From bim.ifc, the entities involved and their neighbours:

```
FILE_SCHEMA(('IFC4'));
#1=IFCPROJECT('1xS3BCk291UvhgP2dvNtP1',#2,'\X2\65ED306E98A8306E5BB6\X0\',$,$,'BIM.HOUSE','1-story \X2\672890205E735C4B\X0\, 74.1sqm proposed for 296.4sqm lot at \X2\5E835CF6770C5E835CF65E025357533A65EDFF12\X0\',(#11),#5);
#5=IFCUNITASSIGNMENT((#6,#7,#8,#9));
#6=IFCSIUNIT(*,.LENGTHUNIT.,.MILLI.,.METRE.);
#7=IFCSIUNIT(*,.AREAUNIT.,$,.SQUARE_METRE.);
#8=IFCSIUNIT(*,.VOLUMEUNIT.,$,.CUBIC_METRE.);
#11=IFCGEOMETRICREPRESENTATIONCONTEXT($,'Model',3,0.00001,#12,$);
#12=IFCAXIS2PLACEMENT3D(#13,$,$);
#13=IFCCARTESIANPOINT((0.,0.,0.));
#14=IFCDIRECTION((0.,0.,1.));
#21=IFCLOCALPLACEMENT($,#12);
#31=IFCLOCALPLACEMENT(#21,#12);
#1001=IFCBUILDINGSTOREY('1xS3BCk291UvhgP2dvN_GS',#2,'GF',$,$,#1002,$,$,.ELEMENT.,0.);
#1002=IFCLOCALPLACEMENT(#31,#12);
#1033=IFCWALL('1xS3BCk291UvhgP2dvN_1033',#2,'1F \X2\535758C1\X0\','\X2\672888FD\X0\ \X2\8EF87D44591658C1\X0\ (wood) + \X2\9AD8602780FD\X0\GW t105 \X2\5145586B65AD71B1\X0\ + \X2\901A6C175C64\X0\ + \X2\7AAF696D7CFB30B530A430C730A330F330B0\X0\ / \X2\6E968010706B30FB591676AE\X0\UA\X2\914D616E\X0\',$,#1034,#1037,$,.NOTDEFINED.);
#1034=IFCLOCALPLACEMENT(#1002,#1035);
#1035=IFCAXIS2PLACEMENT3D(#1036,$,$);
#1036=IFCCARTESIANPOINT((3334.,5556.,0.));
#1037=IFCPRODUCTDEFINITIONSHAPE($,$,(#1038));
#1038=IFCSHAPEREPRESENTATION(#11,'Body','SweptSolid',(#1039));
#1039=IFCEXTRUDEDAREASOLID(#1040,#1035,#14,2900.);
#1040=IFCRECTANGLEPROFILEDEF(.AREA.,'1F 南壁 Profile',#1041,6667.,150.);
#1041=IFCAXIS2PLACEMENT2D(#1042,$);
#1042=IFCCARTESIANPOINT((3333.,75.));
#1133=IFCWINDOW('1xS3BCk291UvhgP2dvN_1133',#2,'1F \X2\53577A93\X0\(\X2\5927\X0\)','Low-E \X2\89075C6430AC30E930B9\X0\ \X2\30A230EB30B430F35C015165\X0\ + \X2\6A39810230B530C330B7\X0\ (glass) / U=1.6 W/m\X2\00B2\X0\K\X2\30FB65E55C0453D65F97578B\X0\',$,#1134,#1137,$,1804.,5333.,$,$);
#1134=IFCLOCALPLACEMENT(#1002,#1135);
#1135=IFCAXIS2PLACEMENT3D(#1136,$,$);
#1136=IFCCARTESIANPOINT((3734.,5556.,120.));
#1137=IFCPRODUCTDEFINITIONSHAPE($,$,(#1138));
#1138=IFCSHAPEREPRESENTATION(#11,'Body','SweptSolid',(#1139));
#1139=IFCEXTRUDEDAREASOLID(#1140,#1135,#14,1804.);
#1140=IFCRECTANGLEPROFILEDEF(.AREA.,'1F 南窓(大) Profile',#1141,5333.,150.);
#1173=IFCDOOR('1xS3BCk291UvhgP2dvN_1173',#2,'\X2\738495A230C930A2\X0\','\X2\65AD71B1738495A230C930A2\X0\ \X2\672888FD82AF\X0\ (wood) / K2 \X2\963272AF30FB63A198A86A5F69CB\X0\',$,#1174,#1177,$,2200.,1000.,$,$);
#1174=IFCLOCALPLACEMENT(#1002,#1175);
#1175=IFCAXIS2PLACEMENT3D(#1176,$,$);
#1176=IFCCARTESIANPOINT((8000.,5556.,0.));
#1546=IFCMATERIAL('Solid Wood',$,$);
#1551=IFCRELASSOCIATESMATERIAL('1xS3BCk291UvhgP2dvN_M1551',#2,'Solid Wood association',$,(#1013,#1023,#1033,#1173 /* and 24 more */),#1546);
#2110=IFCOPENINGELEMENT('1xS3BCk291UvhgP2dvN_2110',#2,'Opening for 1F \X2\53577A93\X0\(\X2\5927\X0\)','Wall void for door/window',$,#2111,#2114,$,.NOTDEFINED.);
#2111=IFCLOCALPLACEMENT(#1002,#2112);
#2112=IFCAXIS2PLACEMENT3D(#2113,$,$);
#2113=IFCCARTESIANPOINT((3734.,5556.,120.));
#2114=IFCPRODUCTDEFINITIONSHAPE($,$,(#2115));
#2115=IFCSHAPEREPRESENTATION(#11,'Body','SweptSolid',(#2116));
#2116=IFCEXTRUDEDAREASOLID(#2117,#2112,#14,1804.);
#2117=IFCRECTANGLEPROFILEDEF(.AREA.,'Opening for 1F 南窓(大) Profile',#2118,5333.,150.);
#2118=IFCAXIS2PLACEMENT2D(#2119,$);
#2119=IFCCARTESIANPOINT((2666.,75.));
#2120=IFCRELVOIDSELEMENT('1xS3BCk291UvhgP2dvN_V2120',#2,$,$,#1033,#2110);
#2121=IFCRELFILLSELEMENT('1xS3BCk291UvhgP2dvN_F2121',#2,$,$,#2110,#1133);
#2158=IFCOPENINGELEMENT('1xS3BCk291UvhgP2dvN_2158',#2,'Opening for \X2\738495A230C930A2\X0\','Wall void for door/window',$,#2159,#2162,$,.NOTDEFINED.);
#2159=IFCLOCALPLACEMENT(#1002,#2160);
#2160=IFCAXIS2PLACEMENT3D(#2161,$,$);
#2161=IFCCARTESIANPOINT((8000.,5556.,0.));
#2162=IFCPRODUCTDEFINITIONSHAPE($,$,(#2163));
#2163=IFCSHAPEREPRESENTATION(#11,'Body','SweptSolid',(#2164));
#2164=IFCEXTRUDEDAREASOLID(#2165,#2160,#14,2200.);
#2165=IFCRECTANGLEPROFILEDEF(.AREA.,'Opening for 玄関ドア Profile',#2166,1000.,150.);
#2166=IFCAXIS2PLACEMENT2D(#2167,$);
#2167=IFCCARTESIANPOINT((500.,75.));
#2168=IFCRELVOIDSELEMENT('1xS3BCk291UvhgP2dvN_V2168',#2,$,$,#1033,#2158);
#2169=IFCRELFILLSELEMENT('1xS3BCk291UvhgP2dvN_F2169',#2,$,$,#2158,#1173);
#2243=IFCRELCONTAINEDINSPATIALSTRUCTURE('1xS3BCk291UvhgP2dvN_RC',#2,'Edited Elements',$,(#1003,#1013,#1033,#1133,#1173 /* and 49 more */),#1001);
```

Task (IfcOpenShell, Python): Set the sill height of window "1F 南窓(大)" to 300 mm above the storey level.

```python
import numpy as np
import ifcopenshell
import ifcopenshell.api.geometry
import ifcopenshell.geom
import ifcopenshell.util.element
import ifcopenshell.util.placement
import ifcopenshell.util.shape
import ifcopenshell.util.unit

model = ifcopenshell.open("bim.ifc")
unit_scale = ifcopenshell.util.unit.calculate_unit_scale(model)

window = model.by_id(1133)
opening = window.FillsVoids[0].RelatingOpeningElement
storey = ifcopenshell.util.element.get_container(window, ifc_class="IfcBuildingStorey")
level = ifcopenshell.util.placement.get_local_placement(storey.ObjectPlacement)[2, 3]

# The opening's origin need not be at the sill, so measure its lowest point.
shape = ifcopenshell.geom.create_shape(ifcopenshell.geom.settings(), opening)
bottom = ifcopenshell.util.shape.get_shape_bottom_elevation(shape, shape.geometry) / unit_scale
dz = level + 0.3 / unit_scale - bottom

shift = np.array([0.0, 0.0, dz])
# The window is not placed relative to its opening, so move both.
for product in (opening, window):
    matrix = ifcopenshell.util.placement.get_local_placement(product.ObjectPlacement)
    matrix[:3, 3] += shift
    ifcopenshell.api.geometry.edit_object_placement(model, product=product, matrix=matrix, is_si=False)

print(f"moved by {dz * unit_scale:+.3f} m")

model.write("bim_rev.ifc")
```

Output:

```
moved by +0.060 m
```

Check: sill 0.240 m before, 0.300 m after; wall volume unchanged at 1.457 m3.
